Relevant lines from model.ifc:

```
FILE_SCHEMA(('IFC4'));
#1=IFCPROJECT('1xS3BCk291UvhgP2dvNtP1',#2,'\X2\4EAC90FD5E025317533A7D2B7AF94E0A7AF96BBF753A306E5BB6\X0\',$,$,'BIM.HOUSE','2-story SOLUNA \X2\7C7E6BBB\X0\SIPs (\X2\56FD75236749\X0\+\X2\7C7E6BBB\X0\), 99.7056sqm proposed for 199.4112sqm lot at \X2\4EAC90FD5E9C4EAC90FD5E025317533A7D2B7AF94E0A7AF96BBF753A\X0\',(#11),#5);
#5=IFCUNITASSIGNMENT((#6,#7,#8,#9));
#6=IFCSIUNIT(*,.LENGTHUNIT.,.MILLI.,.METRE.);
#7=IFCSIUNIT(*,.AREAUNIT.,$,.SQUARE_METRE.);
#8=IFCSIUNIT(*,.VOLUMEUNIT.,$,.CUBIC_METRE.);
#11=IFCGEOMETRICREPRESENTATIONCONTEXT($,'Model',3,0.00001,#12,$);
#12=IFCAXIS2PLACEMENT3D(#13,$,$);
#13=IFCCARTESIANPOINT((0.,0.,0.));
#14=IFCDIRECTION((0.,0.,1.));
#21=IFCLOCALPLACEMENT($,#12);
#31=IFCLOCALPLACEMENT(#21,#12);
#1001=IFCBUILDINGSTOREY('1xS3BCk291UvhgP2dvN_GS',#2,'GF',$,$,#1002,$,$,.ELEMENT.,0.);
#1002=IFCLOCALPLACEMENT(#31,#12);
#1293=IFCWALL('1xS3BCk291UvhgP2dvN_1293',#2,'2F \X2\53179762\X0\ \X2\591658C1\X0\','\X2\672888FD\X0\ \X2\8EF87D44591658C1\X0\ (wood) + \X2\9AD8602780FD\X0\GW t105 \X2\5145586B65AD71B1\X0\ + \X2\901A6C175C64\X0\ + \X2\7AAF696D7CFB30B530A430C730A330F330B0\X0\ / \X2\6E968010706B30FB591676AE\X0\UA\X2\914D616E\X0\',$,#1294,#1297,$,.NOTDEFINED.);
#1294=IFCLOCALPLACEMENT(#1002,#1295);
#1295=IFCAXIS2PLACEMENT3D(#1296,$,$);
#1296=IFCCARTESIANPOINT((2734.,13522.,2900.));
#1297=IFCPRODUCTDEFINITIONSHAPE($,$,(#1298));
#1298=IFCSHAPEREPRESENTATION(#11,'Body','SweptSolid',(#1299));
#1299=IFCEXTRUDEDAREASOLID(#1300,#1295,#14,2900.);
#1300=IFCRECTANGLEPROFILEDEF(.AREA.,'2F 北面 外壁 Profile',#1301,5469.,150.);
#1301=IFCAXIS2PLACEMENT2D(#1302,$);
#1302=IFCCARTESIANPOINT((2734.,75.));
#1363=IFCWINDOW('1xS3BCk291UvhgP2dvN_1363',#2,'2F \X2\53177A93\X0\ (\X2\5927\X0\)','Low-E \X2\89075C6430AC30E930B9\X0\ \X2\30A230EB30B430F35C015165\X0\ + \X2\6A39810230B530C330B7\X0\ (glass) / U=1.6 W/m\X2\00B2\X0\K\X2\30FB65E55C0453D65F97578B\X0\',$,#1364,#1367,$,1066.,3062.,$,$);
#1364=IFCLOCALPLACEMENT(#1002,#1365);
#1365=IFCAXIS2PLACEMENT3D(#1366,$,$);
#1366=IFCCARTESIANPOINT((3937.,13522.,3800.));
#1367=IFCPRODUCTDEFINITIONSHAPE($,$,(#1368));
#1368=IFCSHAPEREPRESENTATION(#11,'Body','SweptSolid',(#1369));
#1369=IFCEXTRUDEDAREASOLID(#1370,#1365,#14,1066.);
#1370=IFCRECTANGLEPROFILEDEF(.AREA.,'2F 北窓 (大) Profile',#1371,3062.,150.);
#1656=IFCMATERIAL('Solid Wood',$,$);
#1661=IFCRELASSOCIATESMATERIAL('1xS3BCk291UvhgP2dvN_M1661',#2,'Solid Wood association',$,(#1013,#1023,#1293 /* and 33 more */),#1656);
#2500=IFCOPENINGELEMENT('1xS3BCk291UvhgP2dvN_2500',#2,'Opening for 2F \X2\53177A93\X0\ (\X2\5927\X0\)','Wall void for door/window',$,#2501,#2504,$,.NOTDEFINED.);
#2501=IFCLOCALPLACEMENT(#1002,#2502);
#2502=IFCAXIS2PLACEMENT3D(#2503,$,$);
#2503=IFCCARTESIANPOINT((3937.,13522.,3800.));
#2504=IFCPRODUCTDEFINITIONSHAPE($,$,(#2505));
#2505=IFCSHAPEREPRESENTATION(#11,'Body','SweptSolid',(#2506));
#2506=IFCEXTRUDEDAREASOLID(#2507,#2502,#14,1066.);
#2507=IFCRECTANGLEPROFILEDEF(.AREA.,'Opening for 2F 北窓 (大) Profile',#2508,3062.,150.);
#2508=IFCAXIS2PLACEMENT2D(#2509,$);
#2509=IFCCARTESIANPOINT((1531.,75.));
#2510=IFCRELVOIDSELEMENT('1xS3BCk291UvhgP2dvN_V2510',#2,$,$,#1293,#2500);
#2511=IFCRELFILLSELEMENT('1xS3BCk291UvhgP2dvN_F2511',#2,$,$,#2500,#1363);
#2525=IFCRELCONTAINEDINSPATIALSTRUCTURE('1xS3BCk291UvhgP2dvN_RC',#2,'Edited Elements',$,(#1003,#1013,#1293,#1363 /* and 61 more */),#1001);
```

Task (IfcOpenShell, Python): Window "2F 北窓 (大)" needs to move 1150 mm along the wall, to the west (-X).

```python
import ifcopenshell
import ifcopenshell.api.geometry
import ifcopenshell.util.placement

model = ifcopenshell.open("model.ifc")

window = model.by_guid("1xS3BCk291UvhgP2dvN_1363")
opening = window.FillsVoids[0].RelatingOpeningElement
wall = opening.VoidsElements[0].RelatingBuildingElement

wall_matrix = ifcopenshell.util.placement.get_local_placement(wall.ObjectPlacement)
shift = wall_matrix[:3, 0] * -1150.0
before = ifcopenshell.util.placement.get_local_placement(window.ObjectPlacement)[:3, 3].copy()

# The window is not placed relative to its opening, so move both.
for product in (opening, window):
    matrix = ifcopenshell.util.placement.get_local_placement(product.ObjectPlacement)
    matrix[:3, 3] += shift
    ifcopenshell.api.geometry.edit_object_placement(model, product=product, matrix=matrix, is_si=False)

after = ifcopenshell.util.placement.get_local_placement(window.ObjectPlacement)[:3, 3]
print("window moved by", (after - before).round(3) + 0.0)

model.write("model_v2.ifc")
```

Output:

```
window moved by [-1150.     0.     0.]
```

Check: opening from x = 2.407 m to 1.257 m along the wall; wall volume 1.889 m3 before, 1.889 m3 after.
